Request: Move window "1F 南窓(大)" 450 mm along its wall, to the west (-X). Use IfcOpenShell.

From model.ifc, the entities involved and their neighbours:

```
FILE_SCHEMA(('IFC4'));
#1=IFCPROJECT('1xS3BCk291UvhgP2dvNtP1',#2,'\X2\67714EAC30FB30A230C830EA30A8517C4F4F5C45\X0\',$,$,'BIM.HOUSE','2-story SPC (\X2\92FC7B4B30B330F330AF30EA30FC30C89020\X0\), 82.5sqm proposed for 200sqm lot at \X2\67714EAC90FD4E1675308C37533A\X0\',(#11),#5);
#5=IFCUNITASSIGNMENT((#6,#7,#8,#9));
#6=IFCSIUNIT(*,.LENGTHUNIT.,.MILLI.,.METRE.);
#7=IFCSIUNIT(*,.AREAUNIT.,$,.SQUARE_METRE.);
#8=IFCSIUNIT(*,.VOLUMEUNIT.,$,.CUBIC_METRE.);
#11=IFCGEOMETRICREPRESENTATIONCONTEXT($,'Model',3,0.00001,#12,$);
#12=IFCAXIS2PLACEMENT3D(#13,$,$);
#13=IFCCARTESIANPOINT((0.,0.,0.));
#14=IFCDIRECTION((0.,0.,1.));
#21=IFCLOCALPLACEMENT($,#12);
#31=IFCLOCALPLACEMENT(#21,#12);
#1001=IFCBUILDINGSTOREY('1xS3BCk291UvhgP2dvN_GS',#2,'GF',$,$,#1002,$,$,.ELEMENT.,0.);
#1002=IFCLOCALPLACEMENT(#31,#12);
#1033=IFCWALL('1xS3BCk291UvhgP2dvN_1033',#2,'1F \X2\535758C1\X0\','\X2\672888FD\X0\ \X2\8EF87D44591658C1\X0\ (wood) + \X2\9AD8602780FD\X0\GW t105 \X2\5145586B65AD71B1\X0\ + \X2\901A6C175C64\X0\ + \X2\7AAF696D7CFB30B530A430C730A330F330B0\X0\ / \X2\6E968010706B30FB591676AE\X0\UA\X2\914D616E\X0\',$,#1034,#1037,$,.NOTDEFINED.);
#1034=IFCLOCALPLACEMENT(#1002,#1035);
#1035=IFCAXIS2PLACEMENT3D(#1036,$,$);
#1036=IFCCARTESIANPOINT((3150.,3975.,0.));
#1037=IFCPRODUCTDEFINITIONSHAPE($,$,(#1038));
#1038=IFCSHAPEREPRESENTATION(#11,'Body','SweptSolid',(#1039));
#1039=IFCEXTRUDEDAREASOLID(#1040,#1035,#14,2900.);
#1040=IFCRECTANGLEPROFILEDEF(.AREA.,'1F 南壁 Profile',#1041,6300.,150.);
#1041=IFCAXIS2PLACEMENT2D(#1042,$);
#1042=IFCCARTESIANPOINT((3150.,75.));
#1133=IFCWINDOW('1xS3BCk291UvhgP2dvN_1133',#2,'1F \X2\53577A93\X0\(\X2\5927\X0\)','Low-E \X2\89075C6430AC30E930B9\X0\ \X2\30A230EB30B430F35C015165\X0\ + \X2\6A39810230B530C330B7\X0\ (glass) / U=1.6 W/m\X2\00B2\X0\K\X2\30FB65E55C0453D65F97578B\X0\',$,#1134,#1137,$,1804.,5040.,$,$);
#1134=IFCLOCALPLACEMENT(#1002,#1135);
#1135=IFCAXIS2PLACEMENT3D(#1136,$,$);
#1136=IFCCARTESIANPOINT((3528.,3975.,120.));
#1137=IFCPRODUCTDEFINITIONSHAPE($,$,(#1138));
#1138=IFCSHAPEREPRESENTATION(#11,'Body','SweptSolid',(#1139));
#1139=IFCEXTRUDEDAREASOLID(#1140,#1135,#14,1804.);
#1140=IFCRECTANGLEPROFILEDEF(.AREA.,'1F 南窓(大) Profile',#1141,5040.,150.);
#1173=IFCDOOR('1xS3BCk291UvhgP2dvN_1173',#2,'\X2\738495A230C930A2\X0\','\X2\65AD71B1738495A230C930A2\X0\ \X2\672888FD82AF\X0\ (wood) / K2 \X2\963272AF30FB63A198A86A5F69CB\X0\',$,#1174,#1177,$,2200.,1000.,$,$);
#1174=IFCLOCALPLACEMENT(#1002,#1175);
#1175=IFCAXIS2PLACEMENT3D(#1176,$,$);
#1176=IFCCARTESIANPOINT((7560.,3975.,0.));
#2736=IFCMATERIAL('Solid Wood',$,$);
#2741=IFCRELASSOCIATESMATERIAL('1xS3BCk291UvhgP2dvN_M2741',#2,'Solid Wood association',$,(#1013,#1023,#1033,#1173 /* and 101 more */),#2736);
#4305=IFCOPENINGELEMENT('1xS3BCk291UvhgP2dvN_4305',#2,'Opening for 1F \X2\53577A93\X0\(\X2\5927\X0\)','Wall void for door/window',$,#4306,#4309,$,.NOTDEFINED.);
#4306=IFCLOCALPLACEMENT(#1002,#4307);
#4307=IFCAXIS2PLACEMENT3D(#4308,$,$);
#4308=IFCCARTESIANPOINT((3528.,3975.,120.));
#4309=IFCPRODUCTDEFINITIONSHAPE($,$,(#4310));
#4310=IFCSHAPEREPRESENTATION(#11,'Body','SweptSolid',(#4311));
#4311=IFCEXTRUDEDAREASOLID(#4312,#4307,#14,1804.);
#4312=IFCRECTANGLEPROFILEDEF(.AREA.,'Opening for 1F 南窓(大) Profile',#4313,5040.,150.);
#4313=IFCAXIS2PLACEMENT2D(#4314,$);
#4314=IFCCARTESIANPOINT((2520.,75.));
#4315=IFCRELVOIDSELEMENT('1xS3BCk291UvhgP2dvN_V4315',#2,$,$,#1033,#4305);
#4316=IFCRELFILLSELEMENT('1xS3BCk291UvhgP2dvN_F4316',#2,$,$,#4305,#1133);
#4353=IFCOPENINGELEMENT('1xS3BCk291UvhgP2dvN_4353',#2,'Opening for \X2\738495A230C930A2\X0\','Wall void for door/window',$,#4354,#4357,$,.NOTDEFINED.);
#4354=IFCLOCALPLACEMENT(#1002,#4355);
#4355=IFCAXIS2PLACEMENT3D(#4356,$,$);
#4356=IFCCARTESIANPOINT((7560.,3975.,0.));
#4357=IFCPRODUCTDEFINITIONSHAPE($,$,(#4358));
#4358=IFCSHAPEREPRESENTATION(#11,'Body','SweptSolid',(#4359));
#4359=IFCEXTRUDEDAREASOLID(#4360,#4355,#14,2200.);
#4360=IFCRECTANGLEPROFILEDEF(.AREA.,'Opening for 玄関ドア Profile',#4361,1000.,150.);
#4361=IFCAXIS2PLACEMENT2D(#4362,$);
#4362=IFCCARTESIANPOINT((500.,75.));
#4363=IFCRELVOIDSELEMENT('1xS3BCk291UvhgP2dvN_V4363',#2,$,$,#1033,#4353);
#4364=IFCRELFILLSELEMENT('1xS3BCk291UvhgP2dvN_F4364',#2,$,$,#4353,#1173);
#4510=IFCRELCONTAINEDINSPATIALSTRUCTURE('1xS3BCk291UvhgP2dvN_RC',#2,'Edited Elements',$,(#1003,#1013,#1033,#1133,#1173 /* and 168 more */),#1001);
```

```python
import ifcopenshell
import ifcopenshell.api.geometry
import ifcopenshell.util.placement
import ifcopenshell.util.unit

model = ifcopenshell.open("model.ifc")
unit_scale = ifcopenshell.util.unit.calculate_unit_scale(model)

window = model.by_guid("1xS3BCk291UvhgP2dvN_1133")
opening = window.FillsVoids[0].RelatingOpeningElement
wall = opening.VoidsElements[0].RelatingBuildingElement

wall_matrix = ifcopenshell.util.placement.get_local_placement(wall.ObjectPlacement)
shift = wall_matrix[:3, 0] * -0.45 / unit_scale
before = ifcopenshell.util.placement.get_local_placement(window.ObjectPlacement)[:3, 3].copy()

# The window is not placed relative to its opening, so move both.
for product in (opening, window):
    matrix = ifcopenshell.util.placement.get_local_placement(product.ObjectPlacement)
    matrix[:3, 3] += shift
    ifcopenshell.api.geometry.edit_object_placement(model, product=product, matrix=matrix, is_si=False)

after = ifcopenshell.util.placement.get_local_placement(window.ObjectPlacement)[:3, 3]
print("window moved by", (after - before).round(3) + 0.0)

model.write("model_v2.ifc")
```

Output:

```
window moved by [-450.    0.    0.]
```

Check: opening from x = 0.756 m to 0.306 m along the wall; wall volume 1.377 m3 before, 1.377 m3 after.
